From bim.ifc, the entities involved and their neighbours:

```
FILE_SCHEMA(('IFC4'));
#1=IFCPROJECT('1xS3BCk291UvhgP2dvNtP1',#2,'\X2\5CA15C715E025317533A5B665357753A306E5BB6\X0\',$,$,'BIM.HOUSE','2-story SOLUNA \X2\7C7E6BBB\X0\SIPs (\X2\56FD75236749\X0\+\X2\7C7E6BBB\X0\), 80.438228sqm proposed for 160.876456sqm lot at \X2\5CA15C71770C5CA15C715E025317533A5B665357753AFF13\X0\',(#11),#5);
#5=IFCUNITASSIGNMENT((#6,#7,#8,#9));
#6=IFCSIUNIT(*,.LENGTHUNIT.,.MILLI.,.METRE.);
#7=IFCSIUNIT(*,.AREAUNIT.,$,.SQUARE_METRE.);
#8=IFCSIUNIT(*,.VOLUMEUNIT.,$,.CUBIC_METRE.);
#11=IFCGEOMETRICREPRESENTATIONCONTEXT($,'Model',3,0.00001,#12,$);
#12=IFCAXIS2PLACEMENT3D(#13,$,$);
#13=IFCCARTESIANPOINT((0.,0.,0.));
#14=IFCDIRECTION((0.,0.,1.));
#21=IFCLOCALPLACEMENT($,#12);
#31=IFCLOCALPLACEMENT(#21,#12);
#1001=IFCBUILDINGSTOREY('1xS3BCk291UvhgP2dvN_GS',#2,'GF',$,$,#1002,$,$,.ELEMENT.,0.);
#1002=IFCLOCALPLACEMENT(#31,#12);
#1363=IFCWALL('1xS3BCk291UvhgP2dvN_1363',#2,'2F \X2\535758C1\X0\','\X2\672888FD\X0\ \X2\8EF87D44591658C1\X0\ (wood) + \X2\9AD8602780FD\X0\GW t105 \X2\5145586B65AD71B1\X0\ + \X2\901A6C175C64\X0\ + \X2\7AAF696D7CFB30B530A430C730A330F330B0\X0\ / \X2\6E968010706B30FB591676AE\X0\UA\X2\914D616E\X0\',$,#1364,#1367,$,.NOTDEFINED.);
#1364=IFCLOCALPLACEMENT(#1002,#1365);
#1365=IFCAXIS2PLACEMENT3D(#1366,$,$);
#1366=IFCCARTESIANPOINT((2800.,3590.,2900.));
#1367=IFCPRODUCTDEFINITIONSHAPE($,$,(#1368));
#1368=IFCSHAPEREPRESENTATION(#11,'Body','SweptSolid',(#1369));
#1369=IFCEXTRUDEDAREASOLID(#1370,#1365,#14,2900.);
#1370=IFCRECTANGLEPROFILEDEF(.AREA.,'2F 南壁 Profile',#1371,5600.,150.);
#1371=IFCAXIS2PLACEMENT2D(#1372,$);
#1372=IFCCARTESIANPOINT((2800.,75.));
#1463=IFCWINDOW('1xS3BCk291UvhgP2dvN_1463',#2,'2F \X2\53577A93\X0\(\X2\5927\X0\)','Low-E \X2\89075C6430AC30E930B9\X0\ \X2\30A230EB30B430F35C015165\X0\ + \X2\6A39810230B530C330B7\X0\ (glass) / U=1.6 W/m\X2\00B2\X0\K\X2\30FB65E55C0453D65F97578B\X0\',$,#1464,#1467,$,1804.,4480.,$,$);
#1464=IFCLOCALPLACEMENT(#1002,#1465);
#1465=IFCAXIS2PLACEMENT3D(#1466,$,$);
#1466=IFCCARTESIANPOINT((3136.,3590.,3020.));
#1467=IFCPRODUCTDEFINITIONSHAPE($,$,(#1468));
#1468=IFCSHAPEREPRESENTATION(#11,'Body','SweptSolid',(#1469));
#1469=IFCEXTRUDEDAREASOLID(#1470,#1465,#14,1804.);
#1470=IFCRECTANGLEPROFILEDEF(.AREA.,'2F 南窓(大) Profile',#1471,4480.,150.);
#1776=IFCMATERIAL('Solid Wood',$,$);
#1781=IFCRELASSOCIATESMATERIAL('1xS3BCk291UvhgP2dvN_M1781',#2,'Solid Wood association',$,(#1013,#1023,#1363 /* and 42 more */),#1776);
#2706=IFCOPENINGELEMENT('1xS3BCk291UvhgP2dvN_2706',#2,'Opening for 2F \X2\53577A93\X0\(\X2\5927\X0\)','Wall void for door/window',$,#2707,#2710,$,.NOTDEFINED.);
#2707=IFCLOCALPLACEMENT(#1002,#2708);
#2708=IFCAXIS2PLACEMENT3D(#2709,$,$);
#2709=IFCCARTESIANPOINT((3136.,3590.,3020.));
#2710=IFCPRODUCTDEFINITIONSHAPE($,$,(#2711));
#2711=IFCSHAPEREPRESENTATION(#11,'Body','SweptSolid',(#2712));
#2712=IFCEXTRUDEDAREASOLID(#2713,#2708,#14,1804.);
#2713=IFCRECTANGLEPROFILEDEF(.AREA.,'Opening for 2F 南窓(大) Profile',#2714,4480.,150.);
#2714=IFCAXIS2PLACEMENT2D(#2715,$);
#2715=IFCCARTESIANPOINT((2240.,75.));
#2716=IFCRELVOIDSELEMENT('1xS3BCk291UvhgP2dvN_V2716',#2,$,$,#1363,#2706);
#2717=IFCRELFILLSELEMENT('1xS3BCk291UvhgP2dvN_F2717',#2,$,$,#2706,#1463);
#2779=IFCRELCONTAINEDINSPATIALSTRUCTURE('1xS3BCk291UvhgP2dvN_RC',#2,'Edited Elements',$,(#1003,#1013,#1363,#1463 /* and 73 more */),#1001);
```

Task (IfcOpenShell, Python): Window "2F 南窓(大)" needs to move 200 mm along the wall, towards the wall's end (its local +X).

```python
import ifcopenshell
import ifcopenshell.api.geometry
import ifcopenshell.util.placement

model = ifcopenshell.open("bim.ifc")

window = model.by_guid("1xS3BCk291UvhgP2dvN_1463")
opening = window.FillsVoids[0].RelatingOpeningElement
wall = opening.VoidsElements[0].RelatingBuildingElement

wall_matrix = ifcopenshell.util.placement.get_local_placement(wall.ObjectPlacement)
shift = wall_matrix[:3, 0] * 200.0
before = ifcopenshell.util.placement.get_local_placement(window.ObjectPlacement)[:3, 3].copy()

# The window is not placed relative to its opening, so move both.
for product in (opening, window):
    matrix = ifcopenshell.util.placement.get_local_placement(product.ObjectPlacement)
    matrix[:3, 3] += shift
    ifcopenshell.api.geometry.edit_object_placement(model, product=product, matrix=matrix, is_si=False)

after = ifcopenshell.util.placement.get_local_placement(window.ObjectPlacement)[:3, 3]
print("window moved by", (after - before).round(3) + 0.0)

model.write("bim_edited.ifc")
```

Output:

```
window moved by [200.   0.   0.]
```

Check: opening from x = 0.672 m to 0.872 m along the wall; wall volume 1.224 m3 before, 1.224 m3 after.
